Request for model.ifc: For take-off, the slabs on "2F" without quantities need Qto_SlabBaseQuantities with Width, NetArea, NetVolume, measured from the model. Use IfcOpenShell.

First a look at what the model holds.

```python
import ifcopenshell
import ifcopenshell.util.element
import ifcopenshell.util.unit

model = ifcopenshell.open("model.ifc")
print(model.schema)
for unit_type in ("LENGTHUNIT", "AREAUNIT", "VOLUMEUNIT"):
    print(unit_type, ifcopenshell.util.unit.calculate_unit_scale(model, unit_type))
storey = next(s for s in model.by_type("IfcBuildingStorey") if s.Name == "2F")
slabs = [e for e in ifcopenshell.util.element.get_decomposition(storey) if e.is_a("IfcSlab")]
for e in sorted(slabs, key=lambda e: e.id()):
    print(e.id(), e.is_a(), e.Name, list(ifcopenshell.util.element.get_psets(e, qtos_only=True)), sep=" | ")
```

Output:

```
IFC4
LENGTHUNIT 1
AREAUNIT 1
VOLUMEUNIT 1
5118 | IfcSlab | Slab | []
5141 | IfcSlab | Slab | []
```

```python
import ifcopenshell
import ifcopenshell.api.pset
import ifcopenshell.geom
import ifcopenshell.util.element
import ifcopenshell.util.shape
import ifcopenshell.util.unit

model = ifcopenshell.open("model.ifc")
unit_scale = ifcopenshell.util.unit.calculate_unit_scale(model)
area_scale = ifcopenshell.util.unit.calculate_unit_scale(model, "AREAUNIT")
volume_scale = ifcopenshell.util.unit.calculate_unit_scale(model, "VOLUMEUNIT")
settings = ifcopenshell.geom.settings()

storey = next(s for s in model.by_type("IfcBuildingStorey") if s.Name == "2F")
slabs = [e for e in ifcopenshell.util.element.get_decomposition(storey) if e.is_a("IfcSlab")]

for e in sorted(slabs, key=lambda e: e.id()):
    if ifcopenshell.util.element.get_psets(e, qtos_only=True, should_inherit=False):
        continue
    # Geometry comes back in metres, in the element's own axes.
    shape = ifcopenshell.geom.create_shape(settings, e)
    values = {
        "Width": ifcopenshell.util.shape.get_z(shape.geometry) / unit_scale,
        "NetArea": ifcopenshell.util.shape.get_footprint_area(shape.geometry) / area_scale,
        "NetVolume": ifcopenshell.util.shape.get_volume(shape.geometry) / volume_scale,
    }
    qto = ifcopenshell.api.pset.add_qto(model, product=e, name="Qto_SlabBaseQuantities")
    ifcopenshell.api.pset.edit_qto(model, qto=qto, properties=values)
    print(e.id(), {k: round(v, 3) for k, v in values.items()})

model.write("model-out.ifc")
```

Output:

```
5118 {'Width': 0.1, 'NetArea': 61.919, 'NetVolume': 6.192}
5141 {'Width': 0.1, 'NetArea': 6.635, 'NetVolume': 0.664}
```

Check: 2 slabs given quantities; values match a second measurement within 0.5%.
